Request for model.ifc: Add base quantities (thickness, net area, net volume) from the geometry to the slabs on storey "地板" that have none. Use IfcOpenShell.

First a look at what the model holds.

```python
import ifcopenshell
import ifcopenshell.util.element
import ifcopenshell.util.unit

model = ifcopenshell.open("model.ifc")
print(model.schema)
for unit_type in ("LENGTHUNIT", "AREAUNIT", "VOLUMEUNIT"):
    print(unit_type, ifcopenshell.util.unit.calculate_unit_scale(model, unit_type))
storey = next(s for s in model.by_type("IfcBuildingStorey") if s.Name == "地板")
slabs = [e for e in ifcopenshell.util.element.get_decomposition(storey) if e.is_a("IfcSlab")]
for e in sorted(slabs, key=lambda e: e.id()):
    print(e.id(), e.is_a(), e.Name, list(ifcopenshell.util.element.get_psets(e, qtos_only=True)), sep=" | ")
```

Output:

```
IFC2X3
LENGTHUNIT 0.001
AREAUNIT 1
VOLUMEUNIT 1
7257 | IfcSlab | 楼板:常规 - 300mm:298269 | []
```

```python
import ifcopenshell
import ifcopenshell.api.pset
import ifcopenshell.geom
import ifcopenshell.util.element
import ifcopenshell.util.shape
import ifcopenshell.util.unit

model = ifcopenshell.open("model.ifc")
unit_scale = ifcopenshell.util.unit.calculate_unit_scale(model)
area_scale = ifcopenshell.util.unit.calculate_unit_scale(model, "AREAUNIT")
volume_scale = ifcopenshell.util.unit.calculate_unit_scale(model, "VOLUMEUNIT")
settings = ifcopenshell.geom.settings()

storey = next(s for s in model.by_type("IfcBuildingStorey") if s.Name == "地板")
slabs = [e for e in ifcopenshell.util.element.get_decomposition(storey) if e.is_a("IfcSlab")]

for e in sorted(slabs, key=lambda e: e.id()):
    if ifcopenshell.util.element.get_psets(e, qtos_only=True, should_inherit=False):
        continue
    # Geometry comes back in metres, in the element's own axes.
    shape = ifcopenshell.geom.create_shape(settings, e)
    values = {
        "Width": ifcopenshell.util.shape.get_z(shape.geometry) / unit_scale,
        "NetArea": ifcopenshell.util.shape.get_footprint_area(shape.geometry) / area_scale,
        "NetVolume": ifcopenshell.util.shape.get_volume(shape.geometry) / volume_scale,
    }
    qto = ifcopenshell.api.pset.add_qto(model, product=e, name="BaseQuantities")
    ifcopenshell.api.pset.edit_qto(model, qto=qto, properties=values)
    print(e.id(), {k: round(v, 3) for k, v in values.items()})

model.write("model_v2.ifc")
```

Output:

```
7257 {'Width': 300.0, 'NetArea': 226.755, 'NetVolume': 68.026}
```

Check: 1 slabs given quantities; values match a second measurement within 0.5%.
